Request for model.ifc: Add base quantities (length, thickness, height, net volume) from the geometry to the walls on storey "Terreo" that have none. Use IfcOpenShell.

First a look at what the model holds.

```python
import ifcopenshell
import ifcopenshell.util.element
import ifcopenshell.util.unit

model = ifcopenshell.open("model.ifc")
print(model.schema)
for unit_type in ("LENGTHUNIT", "AREAUNIT", "VOLUMEUNIT"):
    print(unit_type, ifcopenshell.util.unit.calculate_unit_scale(model, unit_type))
storey = next(s for s in model.by_type("IfcBuildingStorey") if s.Name == "Terreo")
walls = [e for e in ifcopenshell.util.element.get_decomposition(storey) if e.is_a("IfcWall")]
for e in sorted(walls, key=lambda e: e.id()):
    print(e.id(), e.is_a(), e.Name, list(ifcopenshell.util.element.get_psets(e, qtos_only=True)), sep=" | ")
```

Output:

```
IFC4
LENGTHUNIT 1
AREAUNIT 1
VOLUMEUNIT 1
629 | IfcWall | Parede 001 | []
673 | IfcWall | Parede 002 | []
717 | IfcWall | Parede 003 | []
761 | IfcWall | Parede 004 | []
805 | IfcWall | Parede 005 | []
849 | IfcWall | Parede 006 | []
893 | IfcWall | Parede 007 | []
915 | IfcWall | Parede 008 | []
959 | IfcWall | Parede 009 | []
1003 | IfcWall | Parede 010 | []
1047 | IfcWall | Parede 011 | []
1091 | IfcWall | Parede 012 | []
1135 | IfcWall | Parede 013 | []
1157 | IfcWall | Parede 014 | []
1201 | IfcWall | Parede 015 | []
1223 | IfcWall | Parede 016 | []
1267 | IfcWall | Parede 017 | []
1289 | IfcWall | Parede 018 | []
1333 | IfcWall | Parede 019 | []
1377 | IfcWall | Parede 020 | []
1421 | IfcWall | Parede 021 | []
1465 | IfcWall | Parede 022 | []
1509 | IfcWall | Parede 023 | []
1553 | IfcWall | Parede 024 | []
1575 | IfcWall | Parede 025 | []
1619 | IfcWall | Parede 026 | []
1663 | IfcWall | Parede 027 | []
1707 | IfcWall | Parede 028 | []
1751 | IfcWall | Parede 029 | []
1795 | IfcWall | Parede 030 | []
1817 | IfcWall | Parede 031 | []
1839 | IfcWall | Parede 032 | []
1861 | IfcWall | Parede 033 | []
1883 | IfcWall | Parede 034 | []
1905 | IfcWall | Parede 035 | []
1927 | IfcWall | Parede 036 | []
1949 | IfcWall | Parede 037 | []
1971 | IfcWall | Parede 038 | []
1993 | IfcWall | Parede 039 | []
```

```python
import ifcopenshell
import ifcopenshell.api.pset
import ifcopenshell.geom
import ifcopenshell.util.element
import ifcopenshell.util.shape
import ifcopenshell.util.unit

model = ifcopenshell.open("model.ifc")
unit_scale = ifcopenshell.util.unit.calculate_unit_scale(model)
volume_scale = ifcopenshell.util.unit.calculate_unit_scale(model, "VOLUMEUNIT")
settings = ifcopenshell.geom.settings()

storey = next(s for s in model.by_type("IfcBuildingStorey") if s.Name == "Terreo")
walls = [e for e in ifcopenshell.util.element.get_decomposition(storey) if e.is_a("IfcWall")]

for e in sorted(walls, key=lambda e: e.id()):
    if ifcopenshell.util.element.get_psets(e, qtos_only=True, should_inherit=False):
        continue
    # Geometry comes back in metres, in the element's own axes.
    shape = ifcopenshell.geom.create_shape(settings, e)
    values = {
        "Length": ifcopenshell.util.shape.get_x(shape.geometry) / unit_scale,
        "Width": ifcopenshell.util.shape.get_y(shape.geometry) / unit_scale,
        "Height": ifcopenshell.util.shape.get_z(shape.geometry) / unit_scale,
        "NetVolume": ifcopenshell.util.shape.get_volume(shape.geometry) / volume_scale,
    }
    qto = ifcopenshell.api.pset.add_qto(model, product=e, name="Qto_WallBaseQuantities")
    ifcopenshell.api.pset.edit_qto(model, qto=qto, properties=values)
    print(e.id(), {k: round(v, 3) for k, v in values.items()})

model.write("model_rev.ifc")
```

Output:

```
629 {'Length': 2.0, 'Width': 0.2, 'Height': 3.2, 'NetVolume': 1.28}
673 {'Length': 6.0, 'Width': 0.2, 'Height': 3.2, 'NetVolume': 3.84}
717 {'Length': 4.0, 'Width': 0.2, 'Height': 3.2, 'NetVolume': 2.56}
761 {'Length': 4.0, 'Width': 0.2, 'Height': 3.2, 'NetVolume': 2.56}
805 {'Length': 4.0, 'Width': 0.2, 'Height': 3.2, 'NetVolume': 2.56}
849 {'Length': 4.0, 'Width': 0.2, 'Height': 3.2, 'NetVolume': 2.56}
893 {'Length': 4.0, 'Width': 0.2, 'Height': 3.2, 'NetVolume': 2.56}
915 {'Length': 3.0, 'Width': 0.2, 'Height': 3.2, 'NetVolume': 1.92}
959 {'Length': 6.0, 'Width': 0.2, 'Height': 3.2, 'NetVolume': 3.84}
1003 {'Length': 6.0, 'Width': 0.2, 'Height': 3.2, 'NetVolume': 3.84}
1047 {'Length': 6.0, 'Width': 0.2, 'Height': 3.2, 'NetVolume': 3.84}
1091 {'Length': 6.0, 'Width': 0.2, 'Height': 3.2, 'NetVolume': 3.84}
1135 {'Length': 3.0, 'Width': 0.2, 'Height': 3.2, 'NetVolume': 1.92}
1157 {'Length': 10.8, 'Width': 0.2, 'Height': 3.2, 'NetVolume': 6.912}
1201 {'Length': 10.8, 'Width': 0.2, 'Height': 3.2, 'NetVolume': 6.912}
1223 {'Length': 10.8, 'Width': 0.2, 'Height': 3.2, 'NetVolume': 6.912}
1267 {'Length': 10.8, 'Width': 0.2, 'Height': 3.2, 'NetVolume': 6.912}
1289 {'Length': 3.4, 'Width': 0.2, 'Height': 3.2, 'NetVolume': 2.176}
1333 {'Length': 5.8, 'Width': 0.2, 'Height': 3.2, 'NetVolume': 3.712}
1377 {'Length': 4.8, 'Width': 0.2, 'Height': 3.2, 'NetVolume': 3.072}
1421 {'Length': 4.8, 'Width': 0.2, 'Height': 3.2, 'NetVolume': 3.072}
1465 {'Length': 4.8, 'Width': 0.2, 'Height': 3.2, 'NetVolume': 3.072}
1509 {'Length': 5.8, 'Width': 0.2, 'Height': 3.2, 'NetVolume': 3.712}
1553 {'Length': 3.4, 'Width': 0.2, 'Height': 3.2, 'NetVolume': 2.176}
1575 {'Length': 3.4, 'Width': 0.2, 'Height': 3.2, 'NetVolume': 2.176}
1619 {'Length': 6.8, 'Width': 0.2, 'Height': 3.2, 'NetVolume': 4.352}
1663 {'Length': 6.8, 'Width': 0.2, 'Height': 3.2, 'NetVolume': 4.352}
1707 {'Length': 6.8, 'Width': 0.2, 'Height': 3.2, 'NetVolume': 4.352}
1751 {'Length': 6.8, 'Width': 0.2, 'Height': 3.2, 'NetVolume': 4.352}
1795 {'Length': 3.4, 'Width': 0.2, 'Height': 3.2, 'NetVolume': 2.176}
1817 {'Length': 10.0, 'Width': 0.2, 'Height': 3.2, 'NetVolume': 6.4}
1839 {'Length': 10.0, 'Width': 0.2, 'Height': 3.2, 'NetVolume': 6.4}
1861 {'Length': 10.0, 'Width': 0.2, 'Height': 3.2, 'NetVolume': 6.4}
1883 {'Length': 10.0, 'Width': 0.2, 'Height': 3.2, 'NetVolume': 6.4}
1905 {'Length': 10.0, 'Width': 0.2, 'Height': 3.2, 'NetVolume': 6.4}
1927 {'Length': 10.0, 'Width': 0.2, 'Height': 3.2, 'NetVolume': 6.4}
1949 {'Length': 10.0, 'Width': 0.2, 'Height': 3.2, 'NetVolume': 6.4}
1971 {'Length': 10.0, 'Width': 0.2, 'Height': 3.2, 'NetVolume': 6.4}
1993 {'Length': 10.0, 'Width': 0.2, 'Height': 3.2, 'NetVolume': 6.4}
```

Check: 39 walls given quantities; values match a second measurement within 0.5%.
